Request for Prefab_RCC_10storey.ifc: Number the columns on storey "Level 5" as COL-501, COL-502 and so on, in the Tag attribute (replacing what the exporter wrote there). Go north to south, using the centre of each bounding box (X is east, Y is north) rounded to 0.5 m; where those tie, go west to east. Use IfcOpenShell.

First a look at what the model holds.

```python
import ifcopenshell
import ifcopenshell.util.element
import ifcopenshell.util.placement

model = ifcopenshell.open("Prefab_RCC_10storey.ifc")
print(model.schema)
storey = next(s for s in model.by_type("IfcBuildingStorey") if s.Name == "Level 5")
columns = [e for e in ifcopenshell.util.element.get_decomposition(storey) if e.is_a("IfcColumn")]
for e in sorted(columns, key=lambda e: e.id()):
    origin = ifcopenshell.util.placement.get_local_placement(e.ObjectPlacement)[:3, 3]
    print(e.id(), e.Tag, e.Name, origin.round(2) + 0.0, sep=" | ")
```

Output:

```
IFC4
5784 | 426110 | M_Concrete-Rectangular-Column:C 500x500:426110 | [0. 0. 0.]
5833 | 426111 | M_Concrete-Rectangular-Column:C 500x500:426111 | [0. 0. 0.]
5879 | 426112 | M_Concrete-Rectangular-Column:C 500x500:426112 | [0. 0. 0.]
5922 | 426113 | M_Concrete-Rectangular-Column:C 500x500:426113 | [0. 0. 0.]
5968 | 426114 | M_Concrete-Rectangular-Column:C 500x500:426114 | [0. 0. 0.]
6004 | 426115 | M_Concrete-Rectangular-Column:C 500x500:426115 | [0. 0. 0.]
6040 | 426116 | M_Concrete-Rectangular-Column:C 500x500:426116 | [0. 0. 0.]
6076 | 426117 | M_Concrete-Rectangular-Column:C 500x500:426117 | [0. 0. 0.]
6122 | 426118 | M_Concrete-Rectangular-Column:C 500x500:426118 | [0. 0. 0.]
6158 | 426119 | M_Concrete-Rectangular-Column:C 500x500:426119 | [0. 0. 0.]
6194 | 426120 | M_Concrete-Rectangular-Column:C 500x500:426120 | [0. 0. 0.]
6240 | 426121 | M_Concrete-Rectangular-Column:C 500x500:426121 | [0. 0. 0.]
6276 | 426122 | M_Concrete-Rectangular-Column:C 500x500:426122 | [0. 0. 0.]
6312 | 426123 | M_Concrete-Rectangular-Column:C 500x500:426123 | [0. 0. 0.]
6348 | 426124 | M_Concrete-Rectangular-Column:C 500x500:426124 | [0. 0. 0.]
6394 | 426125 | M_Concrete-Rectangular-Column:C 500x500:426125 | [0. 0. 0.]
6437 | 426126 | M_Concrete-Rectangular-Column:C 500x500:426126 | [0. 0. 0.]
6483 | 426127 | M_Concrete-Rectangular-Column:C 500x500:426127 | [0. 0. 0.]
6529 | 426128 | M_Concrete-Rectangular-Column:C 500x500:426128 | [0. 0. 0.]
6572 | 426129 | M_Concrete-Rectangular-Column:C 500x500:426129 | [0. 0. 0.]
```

```python
import ifcopenshell
import ifcopenshell.geom
import ifcopenshell.util.element
import ifcopenshell.util.shape

model = ifcopenshell.open("Prefab_RCC_10storey.ifc")
settings = ifcopenshell.geom.settings()
settings.set("use-world-coords", True)


def centre(element):
    shape = ifcopenshell.geom.create_shape(settings, element)
    return ifcopenshell.util.shape.get_bbox_centroid(shape.geometry)


storey = next(s for s in model.by_type("IfcBuildingStorey") if s.Name == "Level 5")
columns = [e for e in ifcopenshell.util.element.get_decomposition(storey) if e.is_a("IfcColumn")]

# Insertion points can sit at a corner or the storey origin, so sort by the geometry (in metres).
centres = {e: centre(e) for e in columns}
columns.sort(key=lambda e: (-round(centres[e][1] / 0.5), centres[e][0]))

for i, e in enumerate(columns, start=1):
    number = f"COL-5{i:02d}"
    e.Tag = number
    print(e.id(), number)

model.write("Prefab_RCC_10storey_edited.ifc")
```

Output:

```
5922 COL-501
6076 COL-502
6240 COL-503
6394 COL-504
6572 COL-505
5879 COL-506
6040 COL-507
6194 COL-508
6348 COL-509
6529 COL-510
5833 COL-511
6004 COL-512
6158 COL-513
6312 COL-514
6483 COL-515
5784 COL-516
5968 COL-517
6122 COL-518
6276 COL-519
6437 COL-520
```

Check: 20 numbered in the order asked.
